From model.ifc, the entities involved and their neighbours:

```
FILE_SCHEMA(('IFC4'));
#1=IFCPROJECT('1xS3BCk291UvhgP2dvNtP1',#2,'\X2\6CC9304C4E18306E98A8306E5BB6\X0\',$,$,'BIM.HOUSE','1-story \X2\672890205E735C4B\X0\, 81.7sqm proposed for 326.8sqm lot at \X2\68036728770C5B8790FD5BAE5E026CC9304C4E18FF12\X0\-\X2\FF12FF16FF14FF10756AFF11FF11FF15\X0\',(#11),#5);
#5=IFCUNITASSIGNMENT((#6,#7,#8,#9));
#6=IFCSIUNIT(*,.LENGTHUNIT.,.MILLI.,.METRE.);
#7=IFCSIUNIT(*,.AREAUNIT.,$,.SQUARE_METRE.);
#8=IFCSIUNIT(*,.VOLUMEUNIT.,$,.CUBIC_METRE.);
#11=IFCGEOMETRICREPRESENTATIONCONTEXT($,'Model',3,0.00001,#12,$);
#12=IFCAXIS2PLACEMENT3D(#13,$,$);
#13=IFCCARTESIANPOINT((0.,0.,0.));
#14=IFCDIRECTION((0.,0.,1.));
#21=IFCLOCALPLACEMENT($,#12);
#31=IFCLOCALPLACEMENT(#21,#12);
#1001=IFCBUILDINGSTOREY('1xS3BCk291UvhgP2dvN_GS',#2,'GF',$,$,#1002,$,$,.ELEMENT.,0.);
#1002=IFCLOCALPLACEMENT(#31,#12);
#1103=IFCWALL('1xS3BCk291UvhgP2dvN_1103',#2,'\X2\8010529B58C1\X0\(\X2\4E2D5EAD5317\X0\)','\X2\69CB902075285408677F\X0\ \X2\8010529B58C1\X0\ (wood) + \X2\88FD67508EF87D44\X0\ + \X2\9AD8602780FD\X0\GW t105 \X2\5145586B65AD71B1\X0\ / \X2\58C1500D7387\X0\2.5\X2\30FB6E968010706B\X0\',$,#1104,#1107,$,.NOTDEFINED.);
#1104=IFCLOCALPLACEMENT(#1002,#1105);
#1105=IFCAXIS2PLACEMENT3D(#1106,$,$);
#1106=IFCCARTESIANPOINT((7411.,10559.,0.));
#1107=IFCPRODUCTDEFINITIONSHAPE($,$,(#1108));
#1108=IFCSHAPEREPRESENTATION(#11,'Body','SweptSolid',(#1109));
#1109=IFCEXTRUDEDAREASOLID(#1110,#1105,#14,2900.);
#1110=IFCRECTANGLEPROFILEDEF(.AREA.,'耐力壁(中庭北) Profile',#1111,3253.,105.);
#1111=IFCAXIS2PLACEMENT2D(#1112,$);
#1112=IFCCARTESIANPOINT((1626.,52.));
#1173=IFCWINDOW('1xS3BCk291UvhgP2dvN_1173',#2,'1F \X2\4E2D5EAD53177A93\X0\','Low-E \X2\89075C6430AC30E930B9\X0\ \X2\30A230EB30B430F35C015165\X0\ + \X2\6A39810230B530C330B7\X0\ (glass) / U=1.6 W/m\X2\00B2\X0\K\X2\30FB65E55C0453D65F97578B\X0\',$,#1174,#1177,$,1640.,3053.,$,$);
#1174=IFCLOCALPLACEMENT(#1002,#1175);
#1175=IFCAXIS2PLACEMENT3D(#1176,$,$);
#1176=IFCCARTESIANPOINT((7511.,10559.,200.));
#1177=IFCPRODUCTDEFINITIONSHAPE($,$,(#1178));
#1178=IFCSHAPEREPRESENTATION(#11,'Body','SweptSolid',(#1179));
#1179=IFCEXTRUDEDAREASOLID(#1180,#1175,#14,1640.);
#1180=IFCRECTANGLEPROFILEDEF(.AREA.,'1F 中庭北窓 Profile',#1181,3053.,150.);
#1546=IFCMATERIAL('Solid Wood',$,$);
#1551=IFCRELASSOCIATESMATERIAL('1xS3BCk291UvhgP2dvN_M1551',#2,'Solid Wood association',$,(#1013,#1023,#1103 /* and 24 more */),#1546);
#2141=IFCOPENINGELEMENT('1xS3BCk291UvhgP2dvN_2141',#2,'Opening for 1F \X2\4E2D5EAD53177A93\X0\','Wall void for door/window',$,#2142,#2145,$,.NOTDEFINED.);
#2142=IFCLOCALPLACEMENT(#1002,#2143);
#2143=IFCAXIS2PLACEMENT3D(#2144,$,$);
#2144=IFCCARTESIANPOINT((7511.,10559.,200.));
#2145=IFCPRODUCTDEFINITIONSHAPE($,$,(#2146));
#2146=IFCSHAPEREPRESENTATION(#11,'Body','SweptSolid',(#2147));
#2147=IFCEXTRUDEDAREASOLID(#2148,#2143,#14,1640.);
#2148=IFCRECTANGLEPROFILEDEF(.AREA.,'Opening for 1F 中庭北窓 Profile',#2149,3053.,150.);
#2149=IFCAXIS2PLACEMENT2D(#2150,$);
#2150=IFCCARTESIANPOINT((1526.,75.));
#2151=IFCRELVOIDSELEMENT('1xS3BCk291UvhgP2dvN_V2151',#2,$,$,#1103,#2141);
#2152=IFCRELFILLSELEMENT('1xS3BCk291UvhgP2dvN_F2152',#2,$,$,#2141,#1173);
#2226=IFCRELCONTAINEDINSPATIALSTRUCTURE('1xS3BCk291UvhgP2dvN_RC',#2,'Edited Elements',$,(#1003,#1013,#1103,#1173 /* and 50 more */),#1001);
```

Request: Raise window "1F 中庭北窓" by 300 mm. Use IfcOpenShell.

```python
import numpy as np
import ifcopenshell
import ifcopenshell.api.geometry
import ifcopenshell.util.placement
import ifcopenshell.util.unit

model = ifcopenshell.open("model.ifc")
unit_scale = ifcopenshell.util.unit.calculate_unit_scale(model)

window = model.by_guid("1xS3BCk291UvhgP2dvN_1173")
opening = window.FillsVoids[0].RelatingOpeningElement
dz = 0.3 / unit_scale

shift = np.array([0.0, 0.0, dz])
# The window is not placed relative to its opening, so move both.
for product in (opening, window):
    matrix = ifcopenshell.util.placement.get_local_placement(product.ObjectPlacement)
    matrix[:3, 3] += shift
    ifcopenshell.api.geometry.edit_object_placement(model, product=product, matrix=matrix, is_si=False)

print(f"moved by {dz * unit_scale:+.3f} m")

model.write("model_rev.ifc")
```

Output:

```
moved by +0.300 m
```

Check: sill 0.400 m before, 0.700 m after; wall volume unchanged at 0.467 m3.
